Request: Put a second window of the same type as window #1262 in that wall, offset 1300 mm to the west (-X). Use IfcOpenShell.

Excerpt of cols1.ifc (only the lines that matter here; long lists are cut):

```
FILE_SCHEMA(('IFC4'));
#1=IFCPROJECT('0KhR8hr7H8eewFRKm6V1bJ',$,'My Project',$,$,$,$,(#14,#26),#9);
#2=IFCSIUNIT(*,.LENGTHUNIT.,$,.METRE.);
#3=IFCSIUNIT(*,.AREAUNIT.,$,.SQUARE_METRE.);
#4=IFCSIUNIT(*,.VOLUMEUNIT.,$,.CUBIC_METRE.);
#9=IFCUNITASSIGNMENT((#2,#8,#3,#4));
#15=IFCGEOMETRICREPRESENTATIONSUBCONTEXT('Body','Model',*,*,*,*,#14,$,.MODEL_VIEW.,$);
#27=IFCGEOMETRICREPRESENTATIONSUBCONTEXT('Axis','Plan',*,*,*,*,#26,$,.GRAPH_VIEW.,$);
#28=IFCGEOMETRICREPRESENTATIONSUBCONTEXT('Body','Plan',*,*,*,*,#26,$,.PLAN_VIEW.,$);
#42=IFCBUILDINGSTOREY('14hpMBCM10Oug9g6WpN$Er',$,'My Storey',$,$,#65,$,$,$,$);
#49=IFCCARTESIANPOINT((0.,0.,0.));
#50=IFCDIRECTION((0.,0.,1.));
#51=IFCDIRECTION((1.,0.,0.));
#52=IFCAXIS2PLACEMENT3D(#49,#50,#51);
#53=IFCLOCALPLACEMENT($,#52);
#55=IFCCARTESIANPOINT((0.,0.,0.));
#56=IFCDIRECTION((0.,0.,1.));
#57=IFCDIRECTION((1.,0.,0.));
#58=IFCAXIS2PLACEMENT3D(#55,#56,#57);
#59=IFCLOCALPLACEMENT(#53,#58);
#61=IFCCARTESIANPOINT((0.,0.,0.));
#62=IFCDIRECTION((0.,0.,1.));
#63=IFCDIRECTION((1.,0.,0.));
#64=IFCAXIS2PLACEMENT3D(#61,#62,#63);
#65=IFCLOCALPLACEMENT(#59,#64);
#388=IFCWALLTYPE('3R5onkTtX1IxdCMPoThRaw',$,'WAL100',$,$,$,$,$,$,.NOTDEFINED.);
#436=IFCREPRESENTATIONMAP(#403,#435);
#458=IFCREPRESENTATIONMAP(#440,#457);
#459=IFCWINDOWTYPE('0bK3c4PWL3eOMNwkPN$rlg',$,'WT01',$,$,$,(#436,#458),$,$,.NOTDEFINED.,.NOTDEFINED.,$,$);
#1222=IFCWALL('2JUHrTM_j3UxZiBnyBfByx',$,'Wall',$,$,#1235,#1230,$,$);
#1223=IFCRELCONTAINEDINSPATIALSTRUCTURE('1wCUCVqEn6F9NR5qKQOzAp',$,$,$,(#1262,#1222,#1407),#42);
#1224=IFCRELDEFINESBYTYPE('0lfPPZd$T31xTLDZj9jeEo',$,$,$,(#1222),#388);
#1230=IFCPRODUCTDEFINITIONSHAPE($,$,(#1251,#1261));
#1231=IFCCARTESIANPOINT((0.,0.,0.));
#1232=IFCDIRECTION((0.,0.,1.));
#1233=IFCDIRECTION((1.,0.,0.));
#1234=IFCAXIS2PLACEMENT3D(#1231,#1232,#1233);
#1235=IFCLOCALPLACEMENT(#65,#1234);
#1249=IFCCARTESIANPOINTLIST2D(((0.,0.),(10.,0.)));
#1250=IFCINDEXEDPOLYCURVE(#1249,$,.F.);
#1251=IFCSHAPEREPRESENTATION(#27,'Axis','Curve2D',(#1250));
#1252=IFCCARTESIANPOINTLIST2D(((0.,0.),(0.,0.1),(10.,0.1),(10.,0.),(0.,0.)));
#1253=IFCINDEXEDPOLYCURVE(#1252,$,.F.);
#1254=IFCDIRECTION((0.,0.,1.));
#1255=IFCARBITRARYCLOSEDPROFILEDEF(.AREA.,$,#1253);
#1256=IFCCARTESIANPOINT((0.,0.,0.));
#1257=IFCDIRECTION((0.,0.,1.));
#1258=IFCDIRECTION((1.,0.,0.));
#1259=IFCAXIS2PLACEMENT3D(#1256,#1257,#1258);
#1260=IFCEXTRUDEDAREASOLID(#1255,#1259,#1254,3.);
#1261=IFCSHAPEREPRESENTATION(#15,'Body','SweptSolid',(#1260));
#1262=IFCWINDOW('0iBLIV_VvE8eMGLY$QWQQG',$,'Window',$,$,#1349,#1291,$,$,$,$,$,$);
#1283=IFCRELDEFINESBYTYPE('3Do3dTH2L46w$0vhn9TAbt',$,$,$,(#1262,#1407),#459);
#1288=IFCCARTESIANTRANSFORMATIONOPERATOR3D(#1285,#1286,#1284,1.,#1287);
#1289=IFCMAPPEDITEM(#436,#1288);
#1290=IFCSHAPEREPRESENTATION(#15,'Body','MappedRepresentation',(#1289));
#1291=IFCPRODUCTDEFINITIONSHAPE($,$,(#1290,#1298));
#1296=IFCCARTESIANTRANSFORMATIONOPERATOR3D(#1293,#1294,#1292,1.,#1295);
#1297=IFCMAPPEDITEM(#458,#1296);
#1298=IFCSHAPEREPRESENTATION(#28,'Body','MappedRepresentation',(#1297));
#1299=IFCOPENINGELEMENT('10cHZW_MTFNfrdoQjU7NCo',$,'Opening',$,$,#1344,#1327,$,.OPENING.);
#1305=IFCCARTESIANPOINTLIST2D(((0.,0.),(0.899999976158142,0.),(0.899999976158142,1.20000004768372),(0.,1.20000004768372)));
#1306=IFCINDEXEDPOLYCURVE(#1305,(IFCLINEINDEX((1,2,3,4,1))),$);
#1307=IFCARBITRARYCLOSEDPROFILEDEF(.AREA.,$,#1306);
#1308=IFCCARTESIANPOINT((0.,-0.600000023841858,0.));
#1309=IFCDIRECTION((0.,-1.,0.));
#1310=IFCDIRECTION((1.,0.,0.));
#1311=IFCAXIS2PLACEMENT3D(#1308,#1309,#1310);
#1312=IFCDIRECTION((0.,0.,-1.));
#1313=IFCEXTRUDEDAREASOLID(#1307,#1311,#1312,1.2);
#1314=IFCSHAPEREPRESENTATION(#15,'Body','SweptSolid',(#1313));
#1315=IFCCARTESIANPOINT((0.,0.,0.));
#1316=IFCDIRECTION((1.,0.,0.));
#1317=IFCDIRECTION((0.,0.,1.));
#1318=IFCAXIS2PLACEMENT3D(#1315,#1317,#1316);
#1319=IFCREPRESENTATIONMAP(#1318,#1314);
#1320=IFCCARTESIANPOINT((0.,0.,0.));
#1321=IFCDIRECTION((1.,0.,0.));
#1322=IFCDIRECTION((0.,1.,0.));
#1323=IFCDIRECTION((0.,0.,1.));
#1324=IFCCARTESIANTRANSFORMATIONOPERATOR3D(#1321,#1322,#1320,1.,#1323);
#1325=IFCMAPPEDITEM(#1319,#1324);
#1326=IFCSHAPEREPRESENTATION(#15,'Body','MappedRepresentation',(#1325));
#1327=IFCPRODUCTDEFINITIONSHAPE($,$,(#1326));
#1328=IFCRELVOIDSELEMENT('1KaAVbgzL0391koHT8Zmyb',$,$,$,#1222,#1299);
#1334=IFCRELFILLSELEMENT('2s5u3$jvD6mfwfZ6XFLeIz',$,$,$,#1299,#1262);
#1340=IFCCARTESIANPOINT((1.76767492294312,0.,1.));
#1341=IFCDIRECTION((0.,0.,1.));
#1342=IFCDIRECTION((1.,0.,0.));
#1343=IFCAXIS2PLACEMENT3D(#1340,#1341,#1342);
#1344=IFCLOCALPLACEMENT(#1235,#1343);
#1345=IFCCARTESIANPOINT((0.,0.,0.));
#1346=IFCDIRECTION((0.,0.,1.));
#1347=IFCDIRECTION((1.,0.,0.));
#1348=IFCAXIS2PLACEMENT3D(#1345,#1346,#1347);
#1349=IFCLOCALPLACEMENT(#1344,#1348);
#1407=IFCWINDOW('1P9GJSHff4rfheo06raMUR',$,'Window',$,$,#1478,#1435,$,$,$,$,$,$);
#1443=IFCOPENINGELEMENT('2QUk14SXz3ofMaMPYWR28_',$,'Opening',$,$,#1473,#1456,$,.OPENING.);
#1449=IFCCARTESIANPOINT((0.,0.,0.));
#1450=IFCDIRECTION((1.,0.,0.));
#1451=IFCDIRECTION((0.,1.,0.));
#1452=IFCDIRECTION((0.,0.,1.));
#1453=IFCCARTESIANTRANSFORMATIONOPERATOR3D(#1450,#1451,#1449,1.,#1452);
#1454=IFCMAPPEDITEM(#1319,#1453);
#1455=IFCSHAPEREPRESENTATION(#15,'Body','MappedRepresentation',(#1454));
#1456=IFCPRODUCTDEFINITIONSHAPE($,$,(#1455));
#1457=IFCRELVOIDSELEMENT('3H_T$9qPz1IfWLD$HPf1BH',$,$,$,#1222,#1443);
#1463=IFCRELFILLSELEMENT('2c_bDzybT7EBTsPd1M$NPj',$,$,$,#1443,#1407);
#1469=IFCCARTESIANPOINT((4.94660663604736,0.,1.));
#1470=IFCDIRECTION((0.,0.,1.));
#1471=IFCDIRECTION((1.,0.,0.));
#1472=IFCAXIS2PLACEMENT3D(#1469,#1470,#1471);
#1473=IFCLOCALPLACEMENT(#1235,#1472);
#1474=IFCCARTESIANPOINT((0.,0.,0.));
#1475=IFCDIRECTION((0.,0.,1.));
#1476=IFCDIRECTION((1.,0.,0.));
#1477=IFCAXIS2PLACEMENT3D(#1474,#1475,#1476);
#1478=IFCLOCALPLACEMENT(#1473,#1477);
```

```python
import ifcopenshell
import ifcopenshell.api.feature
import ifcopenshell.api.geometry
import ifcopenshell.api.root
import ifcopenshell.geom
import ifcopenshell.util.element
import ifcopenshell.util.placement
import ifcopenshell.util.shape
import ifcopenshell.util.unit

model = ifcopenshell.open("cols1.ifc")
unit_scale = ifcopenshell.util.unit.calculate_unit_scale(model)
settings = ifcopenshell.geom.settings()


def volume(element):
    """Net volume in cubic metres, openings subtracted."""
    shape = ifcopenshell.geom.create_shape(settings, element)
    return ifcopenshell.util.shape.get_volume(shape.geometry)


window = model.by_guid("0iBLIV_VvE8eMGLY$QWQQG")
opening = window.FillsVoids[0].RelatingOpeningElement
wall = opening.VoidsElements[0].RelatingBuildingElement
before = volume(wall)
shift = ifcopenshell.util.placement.get_local_placement(wall.ObjectPlacement)[:3, 0] * -1.3 / unit_scale

# copy_class copies the void relationship, type, container and properties, but no geometry.
new_opening = ifcopenshell.api.root.copy_class(model, product=opening)
new_opening.Representation = ifcopenshell.util.element.copy_deep(
    model, opening.Representation, exclude=["IfcGeometricRepresentationContext", "IfcRepresentationMap"]
)
new_window = ifcopenshell.api.root.copy_class(model, product=window)
new_window.Representation = ifcopenshell.util.element.copy_deep(
    model, window.Representation, exclude=["IfcGeometricRepresentationContext", "IfcRepresentationMap"]
)
ifcopenshell.api.feature.add_filling(model, opening=new_opening, element=new_window)

for old, new in ((opening, new_opening), (window, new_window)):
    matrix = ifcopenshell.util.placement.get_local_placement(old.ObjectPlacement)
    matrix[:3, 3] += shift
    ifcopenshell.api.geometry.edit_object_placement(model, product=new, matrix=matrix, is_si=False)

after = volume(wall)

print(f"wall volume {before:.3f} -> {after:.3f} m3")

model.write("cols1_updated.ifc")
```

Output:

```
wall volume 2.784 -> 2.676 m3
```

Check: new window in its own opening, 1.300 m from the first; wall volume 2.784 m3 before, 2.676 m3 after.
